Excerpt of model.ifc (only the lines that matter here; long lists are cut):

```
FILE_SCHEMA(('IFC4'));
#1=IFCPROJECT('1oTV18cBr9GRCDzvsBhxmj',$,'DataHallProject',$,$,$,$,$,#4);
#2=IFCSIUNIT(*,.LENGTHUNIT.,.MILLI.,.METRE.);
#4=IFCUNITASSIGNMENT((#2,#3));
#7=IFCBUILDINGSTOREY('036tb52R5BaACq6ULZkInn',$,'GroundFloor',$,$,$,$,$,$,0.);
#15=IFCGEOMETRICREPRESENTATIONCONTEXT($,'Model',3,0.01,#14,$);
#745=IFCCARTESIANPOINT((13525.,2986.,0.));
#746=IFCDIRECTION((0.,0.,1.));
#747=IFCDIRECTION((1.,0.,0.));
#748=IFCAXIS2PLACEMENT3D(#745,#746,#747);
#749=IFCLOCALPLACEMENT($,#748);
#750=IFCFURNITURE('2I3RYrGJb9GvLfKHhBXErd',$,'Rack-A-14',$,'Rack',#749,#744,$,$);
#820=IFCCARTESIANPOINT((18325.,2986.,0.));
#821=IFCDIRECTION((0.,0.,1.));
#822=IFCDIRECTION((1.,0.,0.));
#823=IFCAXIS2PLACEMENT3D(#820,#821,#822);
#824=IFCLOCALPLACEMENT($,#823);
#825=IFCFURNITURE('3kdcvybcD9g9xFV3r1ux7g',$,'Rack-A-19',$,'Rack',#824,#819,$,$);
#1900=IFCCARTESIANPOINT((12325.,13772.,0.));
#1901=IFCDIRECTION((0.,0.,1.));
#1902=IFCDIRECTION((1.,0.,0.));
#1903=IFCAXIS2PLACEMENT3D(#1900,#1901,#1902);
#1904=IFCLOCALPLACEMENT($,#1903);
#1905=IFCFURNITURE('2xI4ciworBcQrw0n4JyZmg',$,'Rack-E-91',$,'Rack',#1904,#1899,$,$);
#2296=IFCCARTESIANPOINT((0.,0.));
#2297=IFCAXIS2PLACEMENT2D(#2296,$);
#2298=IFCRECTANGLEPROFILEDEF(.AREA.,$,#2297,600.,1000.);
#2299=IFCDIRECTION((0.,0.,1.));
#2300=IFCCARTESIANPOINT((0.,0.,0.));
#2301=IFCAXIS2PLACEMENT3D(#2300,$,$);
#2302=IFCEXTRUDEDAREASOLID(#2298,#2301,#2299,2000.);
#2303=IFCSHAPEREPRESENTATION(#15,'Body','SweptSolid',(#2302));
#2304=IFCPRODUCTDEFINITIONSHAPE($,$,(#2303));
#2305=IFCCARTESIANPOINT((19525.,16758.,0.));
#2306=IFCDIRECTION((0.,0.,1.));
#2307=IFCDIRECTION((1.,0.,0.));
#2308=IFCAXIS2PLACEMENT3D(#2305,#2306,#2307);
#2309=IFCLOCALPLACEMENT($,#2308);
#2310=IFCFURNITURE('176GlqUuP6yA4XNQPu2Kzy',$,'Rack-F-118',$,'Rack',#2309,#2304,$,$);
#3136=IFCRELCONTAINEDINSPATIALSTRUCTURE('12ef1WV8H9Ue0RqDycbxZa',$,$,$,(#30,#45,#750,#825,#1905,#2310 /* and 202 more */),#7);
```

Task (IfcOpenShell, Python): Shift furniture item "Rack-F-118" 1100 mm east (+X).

```python
import ifcopenshell
import ifcopenshell.api.geometry
import ifcopenshell.util.placement
import ifcopenshell.util.unit

model = ifcopenshell.open("model.ifc")
unit_scale = ifcopenshell.util.unit.calculate_unit_scale(model)

item = model.by_guid("176GlqUuP6yA4XNQPu2Kzy")
matrix = ifcopenshell.util.placement.get_local_placement(item.ObjectPlacement)
matrix[0, 3] += 1.1 / unit_scale
ifcopenshell.api.geometry.edit_object_placement(model, product=item, matrix=matrix, is_si=False)

print(ifcopenshell.util.placement.get_local_placement(item.ObjectPlacement).round(3) + 0.0)

model.write("model_rev.ifc")
```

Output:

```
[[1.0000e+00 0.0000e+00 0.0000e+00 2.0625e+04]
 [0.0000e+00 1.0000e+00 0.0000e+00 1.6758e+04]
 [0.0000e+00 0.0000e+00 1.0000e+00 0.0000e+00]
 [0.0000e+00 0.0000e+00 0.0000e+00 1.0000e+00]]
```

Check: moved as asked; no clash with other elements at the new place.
